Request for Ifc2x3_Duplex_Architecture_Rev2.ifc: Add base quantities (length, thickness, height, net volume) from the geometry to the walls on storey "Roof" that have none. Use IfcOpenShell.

First a look at what the model holds.

```python
import ifcopenshell
import ifcopenshell.util.element
import ifcopenshell.util.unit

model = ifcopenshell.open("Ifc2x3_Duplex_Architecture_Rev2.ifc")
print(model.schema)
for unit_type in ("LENGTHUNIT", "AREAUNIT", "VOLUMEUNIT"):
    print(unit_type, ifcopenshell.util.unit.calculate_unit_scale(model, unit_type))
storey = next(s for s in model.by_type("IfcBuildingStorey") if s.Name == "Roof")
walls = [e for e in ifcopenshell.util.element.get_decomposition(storey) if e.is_a("IfcWall")]
for e in sorted(walls, key=lambda e: e.id()):
    print(e.id(), e.is_a(), e.Name, list(ifcopenshell.util.element.get_psets(e, qtos_only=True)), sep=" | ")
```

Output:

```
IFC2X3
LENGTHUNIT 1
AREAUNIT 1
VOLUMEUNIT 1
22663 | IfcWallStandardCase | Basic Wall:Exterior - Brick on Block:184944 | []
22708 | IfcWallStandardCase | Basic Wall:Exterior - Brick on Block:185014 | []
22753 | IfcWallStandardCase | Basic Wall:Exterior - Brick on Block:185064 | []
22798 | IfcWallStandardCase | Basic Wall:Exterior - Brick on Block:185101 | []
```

```python
import ifcopenshell
import ifcopenshell.api.pset
import ifcopenshell.geom
import ifcopenshell.util.element
import ifcopenshell.util.shape
import ifcopenshell.util.unit

model = ifcopenshell.open("Ifc2x3_Duplex_Architecture_Rev2.ifc")
unit_scale = ifcopenshell.util.unit.calculate_unit_scale(model)
volume_scale = ifcopenshell.util.unit.calculate_unit_scale(model, "VOLUMEUNIT")
settings = ifcopenshell.geom.settings()

storey = next(s for s in model.by_type("IfcBuildingStorey") if s.Name == "Roof")
walls = [e for e in ifcopenshell.util.element.get_decomposition(storey) if e.is_a("IfcWall")]

for e in sorted(walls, key=lambda e: e.id()):
    if ifcopenshell.util.element.get_psets(e, qtos_only=True, should_inherit=False):
        continue
    # Geometry comes back in metres, in the element's own axes.
    shape = ifcopenshell.geom.create_shape(settings, e)
    values = {
        "Length": ifcopenshell.util.shape.get_x(shape.geometry) / unit_scale,
        "Width": ifcopenshell.util.shape.get_y(shape.geometry) / unit_scale,
        "Height": ifcopenshell.util.shape.get_z(shape.geometry) / unit_scale,
        "NetVolume": ifcopenshell.util.shape.get_volume(shape.geometry) / volume_scale,
    }
    qto = ifcopenshell.api.pset.add_qto(model, product=e, name="BaseQuantities")
    ifcopenshell.api.pset.edit_qto(model, qto=qto, properties=values)
    print(e.id(), {k: round(v, 3) for k, v in values.items()})

model.write("Ifc2x3_Duplex_Architecture_Rev2-out.ifc")
```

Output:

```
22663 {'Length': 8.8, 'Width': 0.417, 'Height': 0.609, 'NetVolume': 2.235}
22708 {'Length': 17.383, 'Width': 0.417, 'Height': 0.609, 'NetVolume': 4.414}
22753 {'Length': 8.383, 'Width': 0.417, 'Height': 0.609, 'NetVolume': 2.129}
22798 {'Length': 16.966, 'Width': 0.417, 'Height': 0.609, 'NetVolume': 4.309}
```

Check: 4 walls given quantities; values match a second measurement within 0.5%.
